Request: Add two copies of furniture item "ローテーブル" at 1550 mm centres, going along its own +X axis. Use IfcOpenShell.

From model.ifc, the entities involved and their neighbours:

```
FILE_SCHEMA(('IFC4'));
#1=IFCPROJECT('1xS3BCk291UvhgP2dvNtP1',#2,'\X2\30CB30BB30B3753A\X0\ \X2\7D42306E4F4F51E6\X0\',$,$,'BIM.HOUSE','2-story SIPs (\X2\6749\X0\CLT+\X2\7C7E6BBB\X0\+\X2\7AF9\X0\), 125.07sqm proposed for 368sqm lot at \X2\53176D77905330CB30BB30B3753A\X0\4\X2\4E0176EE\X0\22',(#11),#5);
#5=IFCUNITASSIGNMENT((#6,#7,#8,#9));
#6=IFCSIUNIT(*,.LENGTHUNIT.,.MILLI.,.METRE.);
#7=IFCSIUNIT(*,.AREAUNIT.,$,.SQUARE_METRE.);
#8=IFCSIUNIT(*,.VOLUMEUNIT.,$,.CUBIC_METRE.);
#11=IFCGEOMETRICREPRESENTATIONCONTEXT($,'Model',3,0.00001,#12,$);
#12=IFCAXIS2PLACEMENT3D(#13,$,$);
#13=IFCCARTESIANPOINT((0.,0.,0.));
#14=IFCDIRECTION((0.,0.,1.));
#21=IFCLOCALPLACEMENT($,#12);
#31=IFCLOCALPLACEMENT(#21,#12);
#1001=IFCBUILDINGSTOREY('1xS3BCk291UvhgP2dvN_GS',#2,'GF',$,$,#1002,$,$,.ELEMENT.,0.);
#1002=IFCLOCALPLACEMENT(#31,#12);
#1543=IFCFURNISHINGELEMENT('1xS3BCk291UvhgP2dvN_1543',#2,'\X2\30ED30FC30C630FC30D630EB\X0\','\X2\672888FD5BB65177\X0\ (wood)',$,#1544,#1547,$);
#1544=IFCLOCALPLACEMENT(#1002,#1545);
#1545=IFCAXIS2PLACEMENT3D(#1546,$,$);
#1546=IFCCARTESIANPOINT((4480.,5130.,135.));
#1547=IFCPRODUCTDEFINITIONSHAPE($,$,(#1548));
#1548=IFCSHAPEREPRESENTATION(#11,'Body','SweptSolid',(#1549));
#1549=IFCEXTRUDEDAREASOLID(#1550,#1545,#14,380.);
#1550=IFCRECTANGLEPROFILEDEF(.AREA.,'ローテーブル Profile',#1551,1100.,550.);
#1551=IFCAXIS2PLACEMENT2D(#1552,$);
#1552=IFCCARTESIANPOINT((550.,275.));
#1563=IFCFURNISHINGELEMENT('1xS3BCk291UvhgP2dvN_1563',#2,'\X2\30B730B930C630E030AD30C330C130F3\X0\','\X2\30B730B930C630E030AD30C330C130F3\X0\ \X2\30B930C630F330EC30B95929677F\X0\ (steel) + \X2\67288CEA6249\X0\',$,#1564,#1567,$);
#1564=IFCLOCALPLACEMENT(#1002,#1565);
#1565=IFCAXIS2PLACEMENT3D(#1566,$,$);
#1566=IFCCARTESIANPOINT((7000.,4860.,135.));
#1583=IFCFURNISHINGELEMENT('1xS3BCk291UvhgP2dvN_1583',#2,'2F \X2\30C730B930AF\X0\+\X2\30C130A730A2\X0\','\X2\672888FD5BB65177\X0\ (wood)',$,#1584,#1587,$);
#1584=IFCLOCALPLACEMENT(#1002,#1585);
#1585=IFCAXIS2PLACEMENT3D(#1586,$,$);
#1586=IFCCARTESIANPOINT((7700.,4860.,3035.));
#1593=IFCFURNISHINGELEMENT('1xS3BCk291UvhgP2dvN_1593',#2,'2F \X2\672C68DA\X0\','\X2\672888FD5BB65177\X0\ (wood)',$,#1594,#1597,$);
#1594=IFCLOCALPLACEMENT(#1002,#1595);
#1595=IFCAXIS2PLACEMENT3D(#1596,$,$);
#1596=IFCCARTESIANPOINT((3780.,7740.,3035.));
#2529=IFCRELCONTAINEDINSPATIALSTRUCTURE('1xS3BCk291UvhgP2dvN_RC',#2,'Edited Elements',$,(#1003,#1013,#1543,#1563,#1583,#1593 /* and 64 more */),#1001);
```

```python
import ifcopenshell
import ifcopenshell.api.geometry
import ifcopenshell.api.root
import ifcopenshell.util.element
import ifcopenshell.util.placement

model = ifcopenshell.open("model.ifc")


def reuse_history(source, copy):
    """copy_class also copies each property set's owner history, people and application; keep the originals."""
    for rel in copy.IsDefinedBy:
        if rel.is_a("IfcRelDefinesByProperties") and (history := rel.RelatingPropertyDefinition.OwnerHistory):
            rel.RelatingPropertyDefinition.OwnerHistory = source.OwnerHistory
            ifcopenshell.util.element.remove_deep2(model, history)


source = model.by_guid("1xS3BCk291UvhgP2dvN_1543")
base = ifcopenshell.util.placement.get_local_placement(source.ObjectPlacement)
step = base[:3, 0] * 1550.0

for i in range(1, 3):
    copy = ifcopenshell.api.root.copy_class(model, product=source)
    copy.Representation = ifcopenshell.util.element.copy_deep(
        model, source.Representation, exclude=["IfcGeometricRepresentationContext", "IfcRepresentationMap"]
    )
    reuse_history(source, copy)
    matrix = base.copy()
    matrix[:3, 3] += i * step
    print("added at", matrix[:3, 3].round(3) + 0.0)
    ifcopenshell.api.geometry.edit_object_placement(model, product=copy, matrix=matrix, is_si=False)

model.write("model_v2.ifc")
```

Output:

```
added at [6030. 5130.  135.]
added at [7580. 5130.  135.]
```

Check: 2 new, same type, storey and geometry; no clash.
